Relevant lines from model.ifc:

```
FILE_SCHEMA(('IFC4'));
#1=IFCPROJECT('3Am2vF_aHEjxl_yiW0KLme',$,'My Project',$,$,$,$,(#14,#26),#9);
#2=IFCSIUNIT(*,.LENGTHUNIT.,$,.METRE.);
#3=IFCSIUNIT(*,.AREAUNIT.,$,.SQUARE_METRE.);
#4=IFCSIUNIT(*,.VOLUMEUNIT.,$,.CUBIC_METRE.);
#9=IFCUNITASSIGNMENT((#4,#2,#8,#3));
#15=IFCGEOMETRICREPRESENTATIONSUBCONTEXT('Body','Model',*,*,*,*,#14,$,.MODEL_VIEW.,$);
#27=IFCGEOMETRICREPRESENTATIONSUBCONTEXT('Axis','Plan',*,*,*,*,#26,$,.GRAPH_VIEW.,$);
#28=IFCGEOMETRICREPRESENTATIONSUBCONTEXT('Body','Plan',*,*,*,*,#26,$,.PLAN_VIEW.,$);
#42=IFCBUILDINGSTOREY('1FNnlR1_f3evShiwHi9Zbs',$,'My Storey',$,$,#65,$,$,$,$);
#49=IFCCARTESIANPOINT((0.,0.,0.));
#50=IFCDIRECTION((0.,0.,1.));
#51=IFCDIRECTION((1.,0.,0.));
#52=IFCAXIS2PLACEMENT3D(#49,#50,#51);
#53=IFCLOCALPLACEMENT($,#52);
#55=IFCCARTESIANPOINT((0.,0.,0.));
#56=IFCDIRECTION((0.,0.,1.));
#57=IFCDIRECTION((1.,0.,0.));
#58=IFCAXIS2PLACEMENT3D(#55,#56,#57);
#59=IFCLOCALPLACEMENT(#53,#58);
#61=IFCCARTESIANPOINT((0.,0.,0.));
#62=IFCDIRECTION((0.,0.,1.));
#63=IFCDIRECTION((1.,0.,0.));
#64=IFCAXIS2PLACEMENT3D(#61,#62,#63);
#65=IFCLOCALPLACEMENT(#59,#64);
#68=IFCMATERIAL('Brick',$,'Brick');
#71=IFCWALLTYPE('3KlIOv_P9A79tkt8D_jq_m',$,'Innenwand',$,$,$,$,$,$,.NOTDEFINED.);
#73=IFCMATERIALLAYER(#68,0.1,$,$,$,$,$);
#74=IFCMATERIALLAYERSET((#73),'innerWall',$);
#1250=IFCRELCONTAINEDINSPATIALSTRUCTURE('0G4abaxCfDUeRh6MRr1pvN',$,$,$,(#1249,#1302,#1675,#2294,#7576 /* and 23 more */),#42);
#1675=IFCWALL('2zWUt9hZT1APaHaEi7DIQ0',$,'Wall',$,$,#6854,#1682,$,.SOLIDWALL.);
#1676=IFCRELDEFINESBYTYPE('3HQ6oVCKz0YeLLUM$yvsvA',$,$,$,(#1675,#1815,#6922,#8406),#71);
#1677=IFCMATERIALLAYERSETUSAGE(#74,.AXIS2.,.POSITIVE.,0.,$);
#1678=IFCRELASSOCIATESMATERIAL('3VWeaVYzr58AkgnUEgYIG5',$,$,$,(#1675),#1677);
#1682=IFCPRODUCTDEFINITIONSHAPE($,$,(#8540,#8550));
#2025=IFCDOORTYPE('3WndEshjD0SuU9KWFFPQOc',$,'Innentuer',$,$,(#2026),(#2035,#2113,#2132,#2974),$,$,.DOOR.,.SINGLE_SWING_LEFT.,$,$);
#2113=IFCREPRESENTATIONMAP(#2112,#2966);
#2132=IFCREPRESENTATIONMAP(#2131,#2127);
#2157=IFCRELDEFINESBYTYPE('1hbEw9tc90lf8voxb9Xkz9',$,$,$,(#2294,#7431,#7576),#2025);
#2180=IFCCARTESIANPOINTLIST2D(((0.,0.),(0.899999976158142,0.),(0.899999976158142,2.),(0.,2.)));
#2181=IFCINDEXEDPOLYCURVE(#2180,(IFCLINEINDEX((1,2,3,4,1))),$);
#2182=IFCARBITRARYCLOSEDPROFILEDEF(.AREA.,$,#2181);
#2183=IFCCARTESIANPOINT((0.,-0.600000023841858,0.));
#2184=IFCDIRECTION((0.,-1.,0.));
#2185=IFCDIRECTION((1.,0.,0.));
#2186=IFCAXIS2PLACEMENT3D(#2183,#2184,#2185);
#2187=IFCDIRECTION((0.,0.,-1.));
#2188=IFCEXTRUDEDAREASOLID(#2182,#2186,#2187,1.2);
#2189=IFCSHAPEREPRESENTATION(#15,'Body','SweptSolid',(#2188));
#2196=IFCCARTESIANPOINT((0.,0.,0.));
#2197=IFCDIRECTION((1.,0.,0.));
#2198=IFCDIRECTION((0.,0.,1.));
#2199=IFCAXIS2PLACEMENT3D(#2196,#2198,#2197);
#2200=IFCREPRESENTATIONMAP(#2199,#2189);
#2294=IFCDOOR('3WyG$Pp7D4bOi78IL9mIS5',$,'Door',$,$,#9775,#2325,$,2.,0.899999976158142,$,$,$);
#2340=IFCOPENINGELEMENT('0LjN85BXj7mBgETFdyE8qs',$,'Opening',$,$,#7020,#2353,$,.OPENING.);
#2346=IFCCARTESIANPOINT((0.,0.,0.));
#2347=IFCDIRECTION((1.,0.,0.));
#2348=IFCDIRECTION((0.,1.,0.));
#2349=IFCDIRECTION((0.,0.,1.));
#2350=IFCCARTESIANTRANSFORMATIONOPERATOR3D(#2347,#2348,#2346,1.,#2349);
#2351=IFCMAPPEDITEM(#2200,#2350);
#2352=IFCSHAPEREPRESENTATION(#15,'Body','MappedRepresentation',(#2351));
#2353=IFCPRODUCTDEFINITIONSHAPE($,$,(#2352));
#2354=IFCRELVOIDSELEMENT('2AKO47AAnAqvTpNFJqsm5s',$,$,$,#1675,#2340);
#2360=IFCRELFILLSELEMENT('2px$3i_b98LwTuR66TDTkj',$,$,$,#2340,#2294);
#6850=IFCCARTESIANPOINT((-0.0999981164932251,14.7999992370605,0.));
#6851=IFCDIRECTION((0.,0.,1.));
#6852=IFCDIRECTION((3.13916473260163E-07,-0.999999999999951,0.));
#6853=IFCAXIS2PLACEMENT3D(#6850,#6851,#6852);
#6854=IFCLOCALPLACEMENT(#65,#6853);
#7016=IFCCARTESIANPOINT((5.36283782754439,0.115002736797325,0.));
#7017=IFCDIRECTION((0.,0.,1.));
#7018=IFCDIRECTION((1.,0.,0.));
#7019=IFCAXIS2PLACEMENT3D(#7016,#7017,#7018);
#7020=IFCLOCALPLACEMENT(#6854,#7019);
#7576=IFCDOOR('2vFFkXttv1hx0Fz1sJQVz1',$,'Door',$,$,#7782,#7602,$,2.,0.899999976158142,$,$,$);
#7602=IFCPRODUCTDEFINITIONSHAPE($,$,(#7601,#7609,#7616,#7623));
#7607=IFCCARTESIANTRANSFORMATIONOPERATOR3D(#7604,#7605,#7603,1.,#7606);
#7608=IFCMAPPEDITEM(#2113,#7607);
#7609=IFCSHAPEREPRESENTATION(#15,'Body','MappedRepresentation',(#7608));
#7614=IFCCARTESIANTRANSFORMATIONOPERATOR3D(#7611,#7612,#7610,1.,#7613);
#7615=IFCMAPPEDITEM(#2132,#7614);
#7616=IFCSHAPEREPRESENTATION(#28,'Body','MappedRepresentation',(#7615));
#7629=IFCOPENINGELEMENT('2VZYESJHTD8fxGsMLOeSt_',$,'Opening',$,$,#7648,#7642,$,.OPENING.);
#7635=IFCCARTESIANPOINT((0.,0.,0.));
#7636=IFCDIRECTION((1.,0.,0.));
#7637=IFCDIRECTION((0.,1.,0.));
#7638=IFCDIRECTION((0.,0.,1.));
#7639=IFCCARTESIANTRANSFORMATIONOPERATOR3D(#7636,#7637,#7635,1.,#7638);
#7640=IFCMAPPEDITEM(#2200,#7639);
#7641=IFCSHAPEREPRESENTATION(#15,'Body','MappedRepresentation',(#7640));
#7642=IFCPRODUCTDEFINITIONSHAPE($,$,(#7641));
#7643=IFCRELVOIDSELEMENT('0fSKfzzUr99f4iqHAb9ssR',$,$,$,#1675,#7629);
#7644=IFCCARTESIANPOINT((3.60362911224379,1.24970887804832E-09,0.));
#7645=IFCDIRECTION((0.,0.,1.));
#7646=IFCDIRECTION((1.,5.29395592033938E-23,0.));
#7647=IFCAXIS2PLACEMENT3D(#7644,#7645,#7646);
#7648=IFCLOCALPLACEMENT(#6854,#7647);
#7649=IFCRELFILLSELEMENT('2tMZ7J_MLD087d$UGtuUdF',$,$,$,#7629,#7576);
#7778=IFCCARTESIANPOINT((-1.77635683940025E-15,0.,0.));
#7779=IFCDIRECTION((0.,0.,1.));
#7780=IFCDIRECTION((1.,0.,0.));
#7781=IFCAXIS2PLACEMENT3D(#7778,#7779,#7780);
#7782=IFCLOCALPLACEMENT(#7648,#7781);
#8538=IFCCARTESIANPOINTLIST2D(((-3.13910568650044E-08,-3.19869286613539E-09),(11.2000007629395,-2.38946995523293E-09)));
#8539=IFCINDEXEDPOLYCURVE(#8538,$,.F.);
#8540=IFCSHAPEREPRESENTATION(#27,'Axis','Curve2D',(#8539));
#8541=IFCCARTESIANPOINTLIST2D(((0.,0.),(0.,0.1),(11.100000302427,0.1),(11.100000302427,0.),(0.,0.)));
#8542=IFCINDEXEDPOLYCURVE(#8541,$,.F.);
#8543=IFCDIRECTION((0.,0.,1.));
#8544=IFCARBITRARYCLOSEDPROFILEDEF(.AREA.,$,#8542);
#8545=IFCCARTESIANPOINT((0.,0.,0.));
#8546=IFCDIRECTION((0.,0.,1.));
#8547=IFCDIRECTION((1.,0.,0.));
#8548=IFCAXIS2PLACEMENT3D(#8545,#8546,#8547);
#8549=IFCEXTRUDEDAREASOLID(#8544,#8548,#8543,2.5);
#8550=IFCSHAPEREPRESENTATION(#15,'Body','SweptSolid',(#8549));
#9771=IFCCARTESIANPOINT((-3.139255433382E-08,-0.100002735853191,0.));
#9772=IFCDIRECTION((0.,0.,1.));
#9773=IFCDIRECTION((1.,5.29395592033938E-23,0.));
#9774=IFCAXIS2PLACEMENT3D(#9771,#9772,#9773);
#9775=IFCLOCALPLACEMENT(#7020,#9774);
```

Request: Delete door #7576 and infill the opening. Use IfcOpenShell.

```python
import ifcopenshell
import ifcopenshell.api.feature
import ifcopenshell.api.root
import ifcopenshell.geom
import ifcopenshell.util.shape

model = ifcopenshell.open("model.ifc")
settings = ifcopenshell.geom.settings()


def volume(element):
    """Net volume in cubic metres, openings subtracted."""
    shape = ifcopenshell.geom.create_shape(settings, element)
    return ifcopenshell.util.shape.get_volume(shape.geometry)


door = model.by_id(7576)
opening = door.FillsVoids[0].RelatingOpeningElement
wall = opening.VoidsElements[0].RelatingBuildingElement
before = volume(wall)

ifcopenshell.api.root.remove_product(model, product=door)
ifcopenshell.api.feature.remove_feature(model, feature=opening)

after = volume(wall)

print(f"wall volume {before:.3f} -> {after:.3f} m3")

model.write("model_v2.ifc")
```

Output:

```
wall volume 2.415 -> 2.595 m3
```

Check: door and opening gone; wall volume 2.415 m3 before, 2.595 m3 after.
